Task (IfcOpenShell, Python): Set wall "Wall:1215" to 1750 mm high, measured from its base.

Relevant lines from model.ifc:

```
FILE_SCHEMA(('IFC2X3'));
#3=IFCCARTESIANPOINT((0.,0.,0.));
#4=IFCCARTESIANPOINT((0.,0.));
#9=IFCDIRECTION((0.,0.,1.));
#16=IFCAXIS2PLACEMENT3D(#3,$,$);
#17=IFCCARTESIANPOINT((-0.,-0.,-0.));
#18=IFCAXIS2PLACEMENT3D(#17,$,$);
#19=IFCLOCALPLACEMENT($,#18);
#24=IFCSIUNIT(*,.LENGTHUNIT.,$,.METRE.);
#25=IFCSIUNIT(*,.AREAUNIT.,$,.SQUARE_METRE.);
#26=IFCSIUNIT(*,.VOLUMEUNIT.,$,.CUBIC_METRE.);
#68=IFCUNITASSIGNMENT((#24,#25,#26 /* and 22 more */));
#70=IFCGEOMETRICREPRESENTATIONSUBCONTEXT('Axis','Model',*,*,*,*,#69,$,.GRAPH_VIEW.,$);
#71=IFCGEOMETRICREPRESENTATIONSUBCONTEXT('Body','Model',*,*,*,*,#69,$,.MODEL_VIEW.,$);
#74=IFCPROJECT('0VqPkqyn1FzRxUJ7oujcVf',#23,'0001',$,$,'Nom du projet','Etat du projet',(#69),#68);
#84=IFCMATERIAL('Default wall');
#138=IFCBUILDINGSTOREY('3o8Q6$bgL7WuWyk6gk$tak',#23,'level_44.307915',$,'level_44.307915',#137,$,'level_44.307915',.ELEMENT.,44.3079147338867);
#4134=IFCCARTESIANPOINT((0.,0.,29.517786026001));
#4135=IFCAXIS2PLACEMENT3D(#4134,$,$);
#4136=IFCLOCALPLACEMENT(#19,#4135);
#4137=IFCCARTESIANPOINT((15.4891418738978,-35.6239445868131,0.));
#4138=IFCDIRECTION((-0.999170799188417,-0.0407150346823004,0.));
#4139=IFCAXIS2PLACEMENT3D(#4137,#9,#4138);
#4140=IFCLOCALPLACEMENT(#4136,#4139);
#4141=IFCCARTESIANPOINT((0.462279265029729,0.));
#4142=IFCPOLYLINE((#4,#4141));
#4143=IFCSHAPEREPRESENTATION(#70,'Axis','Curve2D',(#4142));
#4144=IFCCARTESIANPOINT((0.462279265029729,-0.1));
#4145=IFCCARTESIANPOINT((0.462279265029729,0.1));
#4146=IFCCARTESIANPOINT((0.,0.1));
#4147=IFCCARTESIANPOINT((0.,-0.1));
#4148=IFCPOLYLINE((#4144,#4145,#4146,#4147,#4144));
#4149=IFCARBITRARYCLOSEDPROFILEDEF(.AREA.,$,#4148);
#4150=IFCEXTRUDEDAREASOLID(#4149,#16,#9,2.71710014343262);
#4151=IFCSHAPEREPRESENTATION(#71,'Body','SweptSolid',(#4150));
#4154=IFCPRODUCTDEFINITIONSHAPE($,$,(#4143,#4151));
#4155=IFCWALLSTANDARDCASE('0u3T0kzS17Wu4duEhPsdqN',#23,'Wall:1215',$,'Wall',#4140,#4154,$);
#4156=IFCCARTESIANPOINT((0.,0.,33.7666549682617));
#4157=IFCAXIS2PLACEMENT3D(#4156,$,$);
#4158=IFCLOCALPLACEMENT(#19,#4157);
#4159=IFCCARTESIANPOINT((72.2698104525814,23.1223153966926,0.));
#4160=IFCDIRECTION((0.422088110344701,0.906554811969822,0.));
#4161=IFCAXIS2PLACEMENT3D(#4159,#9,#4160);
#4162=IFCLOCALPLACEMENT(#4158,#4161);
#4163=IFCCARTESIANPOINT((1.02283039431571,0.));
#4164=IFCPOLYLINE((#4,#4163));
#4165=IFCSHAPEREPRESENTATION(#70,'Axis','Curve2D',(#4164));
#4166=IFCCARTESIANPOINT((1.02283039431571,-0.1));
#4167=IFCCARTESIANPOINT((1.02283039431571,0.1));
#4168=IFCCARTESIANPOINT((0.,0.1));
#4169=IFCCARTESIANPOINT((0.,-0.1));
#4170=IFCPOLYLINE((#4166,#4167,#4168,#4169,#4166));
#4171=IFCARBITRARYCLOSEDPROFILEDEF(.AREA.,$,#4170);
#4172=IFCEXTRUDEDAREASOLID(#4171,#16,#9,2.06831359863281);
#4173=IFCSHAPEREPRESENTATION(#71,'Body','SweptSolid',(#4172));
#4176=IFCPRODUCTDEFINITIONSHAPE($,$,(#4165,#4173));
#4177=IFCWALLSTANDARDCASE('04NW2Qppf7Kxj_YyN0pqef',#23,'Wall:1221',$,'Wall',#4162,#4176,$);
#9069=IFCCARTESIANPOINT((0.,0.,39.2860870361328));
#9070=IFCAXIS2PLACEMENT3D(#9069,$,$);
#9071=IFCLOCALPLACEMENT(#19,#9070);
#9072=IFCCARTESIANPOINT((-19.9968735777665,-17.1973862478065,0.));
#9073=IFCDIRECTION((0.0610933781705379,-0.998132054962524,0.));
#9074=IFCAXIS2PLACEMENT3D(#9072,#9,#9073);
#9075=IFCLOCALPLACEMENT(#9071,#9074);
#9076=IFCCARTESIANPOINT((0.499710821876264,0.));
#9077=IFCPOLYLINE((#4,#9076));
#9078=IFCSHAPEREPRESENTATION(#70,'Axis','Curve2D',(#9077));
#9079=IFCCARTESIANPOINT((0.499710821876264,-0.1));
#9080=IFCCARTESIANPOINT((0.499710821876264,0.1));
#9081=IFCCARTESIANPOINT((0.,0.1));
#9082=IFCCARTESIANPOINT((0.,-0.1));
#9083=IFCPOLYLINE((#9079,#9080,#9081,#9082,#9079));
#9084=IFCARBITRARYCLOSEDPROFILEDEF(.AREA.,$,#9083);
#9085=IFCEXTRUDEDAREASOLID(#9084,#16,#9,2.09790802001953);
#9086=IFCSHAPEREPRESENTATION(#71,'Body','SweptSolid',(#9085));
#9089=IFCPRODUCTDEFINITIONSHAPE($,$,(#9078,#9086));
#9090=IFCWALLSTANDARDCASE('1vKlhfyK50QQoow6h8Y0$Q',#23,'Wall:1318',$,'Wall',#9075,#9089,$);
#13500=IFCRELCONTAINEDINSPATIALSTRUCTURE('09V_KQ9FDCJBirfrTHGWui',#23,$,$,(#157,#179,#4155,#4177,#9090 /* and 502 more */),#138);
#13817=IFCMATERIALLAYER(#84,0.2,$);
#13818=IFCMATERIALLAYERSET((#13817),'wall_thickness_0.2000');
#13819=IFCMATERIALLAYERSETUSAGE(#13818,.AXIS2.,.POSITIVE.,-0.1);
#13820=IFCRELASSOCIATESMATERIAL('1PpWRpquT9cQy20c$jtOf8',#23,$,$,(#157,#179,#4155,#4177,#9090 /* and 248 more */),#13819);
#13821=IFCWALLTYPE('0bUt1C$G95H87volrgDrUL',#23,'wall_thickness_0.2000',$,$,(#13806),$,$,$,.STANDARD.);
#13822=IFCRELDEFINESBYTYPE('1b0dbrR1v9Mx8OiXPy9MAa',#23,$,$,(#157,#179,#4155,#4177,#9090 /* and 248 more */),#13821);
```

```python
import ifcopenshell
import ifcopenshell.geom
import ifcopenshell.util.representation
import ifcopenshell.util.shape
import ifcopenshell.util.unit

model = ifcopenshell.open("model.ifc")
unit_scale = ifcopenshell.util.unit.calculate_unit_scale(model)
settings = ifcopenshell.geom.settings()


def volume(element):
    """Net volume in cubic metres, openings subtracted."""
    shape = ifcopenshell.geom.create_shape(settings, element)
    return ifcopenshell.util.shape.get_volume(shape.geometry)


wall = model.by_guid("0u3T0kzS17Wu4duEhPsdqN")
before = volume(wall)

body = ifcopenshell.util.representation.get_representation(wall, "Model", "Body")
solid = body.Items[0]
old_height = solid.Depth
solid.Depth = 1.75 / unit_scale
after = volume(wall)

print(f"height {old_height:g} -> {solid.Depth:g}, volume {before:.3f} -> {after:.3f} m3")

model.write("model-out.ifc")
```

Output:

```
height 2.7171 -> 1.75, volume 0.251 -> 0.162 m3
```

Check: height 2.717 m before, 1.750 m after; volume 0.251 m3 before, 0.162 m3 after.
